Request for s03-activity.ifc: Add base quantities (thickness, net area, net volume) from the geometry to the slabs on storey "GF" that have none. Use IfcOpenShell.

First a look at what the model holds.

```python
import ifcopenshell
import ifcopenshell.util.element
import ifcopenshell.util.unit

model = ifcopenshell.open("s03-activity.ifc")
print(model.schema)
for unit_type in ("LENGTHUNIT", "AREAUNIT", "VOLUMEUNIT"):
    print(unit_type, ifcopenshell.util.unit.calculate_unit_scale(model, unit_type))
storey = next(s for s in model.by_type("IfcBuildingStorey") if s.Name == "GF")
slabs = [e for e in ifcopenshell.util.element.get_decomposition(storey) if e.is_a("IfcSlab")]
for e in sorted(slabs, key=lambda e: e.id()):
    print(e.id(), e.is_a(), e.Name, list(ifcopenshell.util.element.get_psets(e, qtos_only=True)), sep=" | ")
```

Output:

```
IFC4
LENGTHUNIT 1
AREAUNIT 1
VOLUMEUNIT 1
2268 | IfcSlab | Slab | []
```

```python
import ifcopenshell
import ifcopenshell.api.pset
import ifcopenshell.geom
import ifcopenshell.util.element
import ifcopenshell.util.shape
import ifcopenshell.util.unit

model = ifcopenshell.open("s03-activity.ifc")
unit_scale = ifcopenshell.util.unit.calculate_unit_scale(model)
area_scale = ifcopenshell.util.unit.calculate_unit_scale(model, "AREAUNIT")
volume_scale = ifcopenshell.util.unit.calculate_unit_scale(model, "VOLUMEUNIT")
settings = ifcopenshell.geom.settings()

storey = next(s for s in model.by_type("IfcBuildingStorey") if s.Name == "GF")
slabs = [e for e in ifcopenshell.util.element.get_decomposition(storey) if e.is_a("IfcSlab")]

for e in sorted(slabs, key=lambda e: e.id()):
    if ifcopenshell.util.element.get_psets(e, qtos_only=True, should_inherit=False):
        continue
    # Geometry comes back in metres, in the element's own axes.
    shape = ifcopenshell.geom.create_shape(settings, e)
    values = {
        "Width": ifcopenshell.util.shape.get_z(shape.geometry) / unit_scale,
        "NetArea": ifcopenshell.util.shape.get_footprint_area(shape.geometry) / area_scale,
        "NetVolume": ifcopenshell.util.shape.get_volume(shape.geometry) / volume_scale,
    }
    qto = ifcopenshell.api.pset.add_qto(model, product=e, name="Qto_SlabBaseQuantities")
    ifcopenshell.api.pset.edit_qto(model, qto=qto, properties=values)
    print(e.id(), {k: round(v, 3) for k, v in values.items()})

model.write("s03-activity_updated.ifc")
```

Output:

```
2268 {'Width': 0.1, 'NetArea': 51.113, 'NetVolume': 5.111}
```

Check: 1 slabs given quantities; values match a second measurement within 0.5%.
